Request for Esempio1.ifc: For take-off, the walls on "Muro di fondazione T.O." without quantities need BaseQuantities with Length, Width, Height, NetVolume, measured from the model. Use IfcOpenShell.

First a look at what the model holds.

```python
import ifcopenshell
import ifcopenshell.util.element
import ifcopenshell.util.unit

model = ifcopenshell.open("Esempio1.ifc")
print(model.schema)
for unit_type in ("LENGTHUNIT", "AREAUNIT", "VOLUMEUNIT"):
    print(unit_type, ifcopenshell.util.unit.calculate_unit_scale(model, unit_type))
storey = next(s for s in model.by_type("IfcBuildingStorey") if s.Name == "Muro di fondazione T.O.")
walls = [e for e in ifcopenshell.util.element.get_decomposition(storey) if e.is_a("IfcWall")]
for e in sorted(walls, key=lambda e: e.id()):
    print(e.id(), e.is_a(), e.Name, list(ifcopenshell.util.element.get_psets(e, qtos_only=True)), sep=" | ")
```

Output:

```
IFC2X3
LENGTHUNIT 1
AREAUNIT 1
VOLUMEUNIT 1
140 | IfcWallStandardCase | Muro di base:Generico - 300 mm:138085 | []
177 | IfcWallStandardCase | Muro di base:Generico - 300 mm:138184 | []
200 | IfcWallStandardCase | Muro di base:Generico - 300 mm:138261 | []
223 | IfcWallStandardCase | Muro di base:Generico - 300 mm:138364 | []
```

```python
import ifcopenshell
import ifcopenshell.api.pset
import ifcopenshell.geom
import ifcopenshell.util.element
import ifcopenshell.util.shape
import ifcopenshell.util.unit

model = ifcopenshell.open("Esempio1.ifc")
unit_scale = ifcopenshell.util.unit.calculate_unit_scale(model)
volume_scale = ifcopenshell.util.unit.calculate_unit_scale(model, "VOLUMEUNIT")
settings = ifcopenshell.geom.settings()

storey = next(s for s in model.by_type("IfcBuildingStorey") if s.Name == "Muro di fondazione T.O.")
walls = [e for e in ifcopenshell.util.element.get_decomposition(storey) if e.is_a("IfcWall")]

for e in sorted(walls, key=lambda e: e.id()):
    if ifcopenshell.util.element.get_psets(e, qtos_only=True, should_inherit=False):
        continue
    # Geometry comes back in metres, in the element's own axes.
    shape = ifcopenshell.geom.create_shape(settings, e)
    values = {
        "Length": ifcopenshell.util.shape.get_x(shape.geometry) / unit_scale,
        "Width": ifcopenshell.util.shape.get_y(shape.geometry) / unit_scale,
        "Height": ifcopenshell.util.shape.get_z(shape.geometry) / unit_scale,
        "NetVolume": ifcopenshell.util.shape.get_volume(shape.geometry) / volume_scale,
    }
    qto = ifcopenshell.api.pset.add_qto(model, product=e, name="BaseQuantities")
    ifcopenshell.api.pset.edit_qto(model, qto=qto, properties=values)
    print(e.id(), {k: round(v, 3) for k, v in values.items()})

model.write("Esempio1_edited.ifc")
```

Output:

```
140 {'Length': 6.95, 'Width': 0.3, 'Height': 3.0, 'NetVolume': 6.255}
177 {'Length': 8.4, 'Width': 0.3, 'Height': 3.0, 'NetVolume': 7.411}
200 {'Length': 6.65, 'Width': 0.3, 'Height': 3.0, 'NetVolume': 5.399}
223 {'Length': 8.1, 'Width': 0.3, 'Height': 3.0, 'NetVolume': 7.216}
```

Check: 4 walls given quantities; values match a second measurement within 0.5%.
